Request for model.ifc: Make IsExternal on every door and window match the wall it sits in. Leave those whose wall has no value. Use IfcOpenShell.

First a look at what the model holds.

```python
import ifcopenshell
import ifcopenshell.util.element

model = ifcopenshell.open("model.ifc")
print(model.schema)
seen = {}
for e in model.by_type("IfcDoor") + model.by_type("IfcWindow"):
    if not e.FillsVoids:
        continue
    host = e.FillsVoids[0].RelatingOpeningElement.VoidsElements[0].RelatingBuildingElement
    own = ifcopenshell.util.element.get_pset(e, f"Pset_{e.is_a()[3:].removesuffix('StandardCase')}Common", "IsExternal")
    wall = ifcopenshell.util.element.get_pset(host, "Pset_WallCommon", "IsExternal")
    seen[e.is_a(), own, wall] = seen.get((e.is_a(), own, wall), 0) + 1
for (cls, own, wall), count in sorted(seen.items(), key=str):
    print(count, cls, "IsExternal:", own, "| host wall:", wall)
```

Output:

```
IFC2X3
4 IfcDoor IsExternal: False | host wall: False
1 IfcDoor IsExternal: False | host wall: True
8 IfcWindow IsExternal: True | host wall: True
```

```python
import ifcopenshell
import ifcopenshell.api.pset
import ifcopenshell.util.element

model = ifcopenshell.open("model.ifc")

count = 0
for ifc_class, pset_name in (("IfcDoor", "Pset_DoorCommon"), ("IfcWindow", "Pset_WindowCommon")):
    for e in model.by_type(ifc_class):
        if not e.FillsVoids:
            continue
        host = e.FillsVoids[0].RelatingOpeningElement.VoidsElements[0].RelatingBuildingElement
        external = ifcopenshell.util.element.get_pset(host, "Pset_WallCommon", "IsExternal")
        if external is None or ifcopenshell.util.element.get_pset(e, pset_name, "IsExternal") == external:
            continue
        pset = ifcopenshell.api.pset.add_pset(model, product=e, name=pset_name)
        ifcopenshell.api.pset.edit_pset(model, pset=pset, properties={"IsExternal": external})
        count += 1

print(count, "updated")

model.write("model_updated.ifc")
```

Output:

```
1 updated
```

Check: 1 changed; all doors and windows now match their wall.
